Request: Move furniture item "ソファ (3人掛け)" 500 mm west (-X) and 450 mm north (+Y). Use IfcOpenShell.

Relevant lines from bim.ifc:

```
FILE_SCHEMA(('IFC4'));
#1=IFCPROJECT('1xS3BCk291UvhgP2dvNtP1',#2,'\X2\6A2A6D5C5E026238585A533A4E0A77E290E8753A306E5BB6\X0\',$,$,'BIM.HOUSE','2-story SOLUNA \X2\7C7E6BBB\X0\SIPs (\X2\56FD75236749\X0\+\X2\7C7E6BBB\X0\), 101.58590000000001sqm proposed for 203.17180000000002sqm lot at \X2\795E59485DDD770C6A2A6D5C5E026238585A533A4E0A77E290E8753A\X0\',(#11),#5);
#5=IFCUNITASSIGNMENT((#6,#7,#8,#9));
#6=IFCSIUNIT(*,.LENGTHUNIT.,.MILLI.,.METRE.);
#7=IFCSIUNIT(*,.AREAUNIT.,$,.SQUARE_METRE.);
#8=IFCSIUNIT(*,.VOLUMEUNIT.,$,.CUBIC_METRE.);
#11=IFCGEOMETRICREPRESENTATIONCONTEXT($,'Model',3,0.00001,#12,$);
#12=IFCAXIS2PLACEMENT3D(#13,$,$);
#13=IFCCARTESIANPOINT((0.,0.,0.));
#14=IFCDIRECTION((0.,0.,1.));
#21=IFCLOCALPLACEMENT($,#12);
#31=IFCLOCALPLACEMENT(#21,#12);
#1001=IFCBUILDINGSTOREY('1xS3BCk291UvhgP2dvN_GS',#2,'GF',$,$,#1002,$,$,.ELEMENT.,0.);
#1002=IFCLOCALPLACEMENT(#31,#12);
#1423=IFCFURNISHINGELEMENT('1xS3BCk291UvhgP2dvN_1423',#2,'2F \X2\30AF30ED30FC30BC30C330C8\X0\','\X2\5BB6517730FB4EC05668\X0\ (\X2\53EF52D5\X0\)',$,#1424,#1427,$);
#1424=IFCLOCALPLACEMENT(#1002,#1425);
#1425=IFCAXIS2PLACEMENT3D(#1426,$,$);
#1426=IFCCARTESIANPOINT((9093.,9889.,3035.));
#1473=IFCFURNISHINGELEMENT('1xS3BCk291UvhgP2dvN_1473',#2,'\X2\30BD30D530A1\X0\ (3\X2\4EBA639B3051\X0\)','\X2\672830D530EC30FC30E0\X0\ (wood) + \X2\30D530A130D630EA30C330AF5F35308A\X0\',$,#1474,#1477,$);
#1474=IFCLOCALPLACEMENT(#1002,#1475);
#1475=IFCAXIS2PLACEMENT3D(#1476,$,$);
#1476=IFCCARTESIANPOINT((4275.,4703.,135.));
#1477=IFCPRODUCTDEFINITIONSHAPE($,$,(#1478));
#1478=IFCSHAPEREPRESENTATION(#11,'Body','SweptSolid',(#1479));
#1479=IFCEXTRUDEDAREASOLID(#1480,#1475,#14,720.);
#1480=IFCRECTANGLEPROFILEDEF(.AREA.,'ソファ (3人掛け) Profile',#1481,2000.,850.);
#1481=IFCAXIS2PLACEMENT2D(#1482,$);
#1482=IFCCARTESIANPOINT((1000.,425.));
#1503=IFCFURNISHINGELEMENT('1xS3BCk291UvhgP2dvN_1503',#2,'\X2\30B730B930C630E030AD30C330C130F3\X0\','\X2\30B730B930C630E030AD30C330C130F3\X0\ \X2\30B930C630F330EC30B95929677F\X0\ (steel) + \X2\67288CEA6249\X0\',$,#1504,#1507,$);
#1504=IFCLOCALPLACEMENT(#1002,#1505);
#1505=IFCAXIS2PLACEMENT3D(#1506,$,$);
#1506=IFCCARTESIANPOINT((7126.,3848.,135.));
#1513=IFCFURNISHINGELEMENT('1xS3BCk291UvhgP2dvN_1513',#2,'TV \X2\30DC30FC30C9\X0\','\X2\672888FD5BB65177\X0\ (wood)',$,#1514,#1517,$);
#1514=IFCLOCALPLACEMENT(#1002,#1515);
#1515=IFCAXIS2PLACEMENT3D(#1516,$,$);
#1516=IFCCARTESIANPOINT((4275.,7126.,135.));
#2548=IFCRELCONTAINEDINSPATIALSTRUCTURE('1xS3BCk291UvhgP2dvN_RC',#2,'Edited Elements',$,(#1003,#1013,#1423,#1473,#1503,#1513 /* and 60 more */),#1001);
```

```python
import ifcopenshell
import ifcopenshell.api.geometry
import ifcopenshell.util.placement
import ifcopenshell.util.unit

model = ifcopenshell.open("bim.ifc")
unit_scale = ifcopenshell.util.unit.calculate_unit_scale(model)

item = model.by_guid("1xS3BCk291UvhgP2dvN_1473")
matrix = ifcopenshell.util.placement.get_local_placement(item.ObjectPlacement)
matrix[0, 3] -= 0.5 / unit_scale
matrix[1, 3] += 0.45 / unit_scale
ifcopenshell.api.geometry.edit_object_placement(model, product=item, matrix=matrix, is_si=False)

print(ifcopenshell.util.placement.get_local_placement(item.ObjectPlacement).round(3) + 0.0)

model.write("bim_v2.ifc")
```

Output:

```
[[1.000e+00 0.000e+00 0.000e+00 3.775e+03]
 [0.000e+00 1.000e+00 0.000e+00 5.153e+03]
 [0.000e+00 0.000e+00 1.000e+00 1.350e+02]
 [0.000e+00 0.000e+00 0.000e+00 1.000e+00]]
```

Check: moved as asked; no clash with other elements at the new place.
